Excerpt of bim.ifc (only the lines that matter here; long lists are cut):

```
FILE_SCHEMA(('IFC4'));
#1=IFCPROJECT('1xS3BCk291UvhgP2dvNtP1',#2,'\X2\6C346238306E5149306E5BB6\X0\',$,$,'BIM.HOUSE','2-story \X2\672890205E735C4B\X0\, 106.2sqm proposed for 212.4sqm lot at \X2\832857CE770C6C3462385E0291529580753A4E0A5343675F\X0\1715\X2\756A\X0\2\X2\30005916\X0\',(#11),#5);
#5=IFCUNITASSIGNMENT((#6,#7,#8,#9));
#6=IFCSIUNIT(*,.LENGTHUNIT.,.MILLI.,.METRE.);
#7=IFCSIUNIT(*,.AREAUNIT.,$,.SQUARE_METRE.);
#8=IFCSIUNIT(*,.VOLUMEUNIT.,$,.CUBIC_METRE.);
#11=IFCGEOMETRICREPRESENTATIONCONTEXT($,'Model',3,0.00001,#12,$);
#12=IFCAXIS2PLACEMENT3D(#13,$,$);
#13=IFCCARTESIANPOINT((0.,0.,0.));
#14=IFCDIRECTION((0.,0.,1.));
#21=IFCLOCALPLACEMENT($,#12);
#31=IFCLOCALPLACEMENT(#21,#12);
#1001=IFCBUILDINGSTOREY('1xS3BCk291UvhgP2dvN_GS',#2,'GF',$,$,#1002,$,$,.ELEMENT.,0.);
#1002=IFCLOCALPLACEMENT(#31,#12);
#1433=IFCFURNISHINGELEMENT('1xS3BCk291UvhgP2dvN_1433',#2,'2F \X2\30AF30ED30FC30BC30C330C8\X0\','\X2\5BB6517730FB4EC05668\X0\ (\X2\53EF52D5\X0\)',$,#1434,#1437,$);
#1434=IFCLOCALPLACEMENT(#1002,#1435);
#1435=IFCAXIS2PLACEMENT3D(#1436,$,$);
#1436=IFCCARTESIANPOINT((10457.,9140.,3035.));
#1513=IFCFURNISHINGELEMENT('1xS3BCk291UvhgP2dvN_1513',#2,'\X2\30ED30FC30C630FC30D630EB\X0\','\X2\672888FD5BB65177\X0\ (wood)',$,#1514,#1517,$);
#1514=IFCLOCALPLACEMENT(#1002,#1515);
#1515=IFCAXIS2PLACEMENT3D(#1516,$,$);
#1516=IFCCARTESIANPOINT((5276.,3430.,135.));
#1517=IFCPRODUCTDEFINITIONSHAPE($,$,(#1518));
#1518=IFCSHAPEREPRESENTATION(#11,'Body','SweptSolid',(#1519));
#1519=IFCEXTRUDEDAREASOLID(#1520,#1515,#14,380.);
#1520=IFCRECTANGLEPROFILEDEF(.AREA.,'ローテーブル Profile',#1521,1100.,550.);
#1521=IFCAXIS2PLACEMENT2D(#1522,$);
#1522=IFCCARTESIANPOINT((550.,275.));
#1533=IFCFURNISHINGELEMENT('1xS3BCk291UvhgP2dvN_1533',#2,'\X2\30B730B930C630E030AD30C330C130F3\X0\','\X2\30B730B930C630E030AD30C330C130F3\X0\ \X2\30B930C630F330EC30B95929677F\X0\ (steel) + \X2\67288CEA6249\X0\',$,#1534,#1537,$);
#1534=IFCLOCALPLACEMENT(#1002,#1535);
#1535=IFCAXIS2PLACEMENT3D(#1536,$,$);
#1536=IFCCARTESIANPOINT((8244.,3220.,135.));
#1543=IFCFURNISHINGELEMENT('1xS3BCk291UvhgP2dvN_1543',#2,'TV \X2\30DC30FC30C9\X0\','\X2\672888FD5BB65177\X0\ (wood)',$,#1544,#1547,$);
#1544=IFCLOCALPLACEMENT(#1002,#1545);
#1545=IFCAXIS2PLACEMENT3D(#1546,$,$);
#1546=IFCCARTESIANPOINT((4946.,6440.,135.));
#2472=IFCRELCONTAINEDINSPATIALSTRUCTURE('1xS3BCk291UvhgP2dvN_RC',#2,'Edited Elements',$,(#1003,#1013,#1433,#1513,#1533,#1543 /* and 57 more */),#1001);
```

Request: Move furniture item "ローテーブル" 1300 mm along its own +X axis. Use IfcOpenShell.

```python
import ifcopenshell
import ifcopenshell.api.geometry
import ifcopenshell.util.placement
import ifcopenshell.util.unit

model = ifcopenshell.open("bim.ifc")
unit_scale = ifcopenshell.util.unit.calculate_unit_scale(model)

item = model.by_id(1513)
matrix = ifcopenshell.util.placement.get_local_placement(item.ObjectPlacement)
matrix[:3, 3] += matrix[:3, 0] * 1.3 / unit_scale
ifcopenshell.api.geometry.edit_object_placement(model, product=item, matrix=matrix, is_si=False)

print(ifcopenshell.util.placement.get_local_placement(item.ObjectPlacement).round(3) + 0.0)

model.write("bim_updated.ifc")
```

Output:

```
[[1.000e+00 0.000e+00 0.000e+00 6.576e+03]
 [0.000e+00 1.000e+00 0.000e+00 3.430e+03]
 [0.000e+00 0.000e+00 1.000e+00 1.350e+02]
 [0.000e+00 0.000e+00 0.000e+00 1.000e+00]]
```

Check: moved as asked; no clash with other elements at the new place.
